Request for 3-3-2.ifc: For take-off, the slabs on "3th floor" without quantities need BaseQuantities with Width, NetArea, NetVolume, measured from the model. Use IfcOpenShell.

First a look at what the model holds.

```python
import ifcopenshell
import ifcopenshell.util.element
import ifcopenshell.util.unit

model = ifcopenshell.open("3-3-2.ifc")
print(model.schema)
for unit_type in ("LENGTHUNIT", "AREAUNIT", "VOLUMEUNIT"):
    print(unit_type, ifcopenshell.util.unit.calculate_unit_scale(model, unit_type))
storey = next(s for s in model.by_type("IfcBuildingStorey") if s.Name == "3th floor")
slabs = [e for e in ifcopenshell.util.element.get_decomposition(storey) if e.is_a("IfcSlab")]
for e in sorted(slabs, key=lambda e: e.id()):
    print(e.id(), e.is_a(), e.Name, list(ifcopenshell.util.element.get_psets(e, qtos_only=True)), sep=" | ")
```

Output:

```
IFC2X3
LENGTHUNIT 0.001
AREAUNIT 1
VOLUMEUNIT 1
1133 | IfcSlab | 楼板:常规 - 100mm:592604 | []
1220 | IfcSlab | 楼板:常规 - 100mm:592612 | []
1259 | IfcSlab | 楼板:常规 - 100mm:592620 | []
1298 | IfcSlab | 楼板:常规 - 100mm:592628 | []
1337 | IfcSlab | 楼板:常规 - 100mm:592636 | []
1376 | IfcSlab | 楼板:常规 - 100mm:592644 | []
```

```python
import ifcopenshell
import ifcopenshell.api.pset
import ifcopenshell.geom
import ifcopenshell.util.element
import ifcopenshell.util.shape
import ifcopenshell.util.unit

model = ifcopenshell.open("3-3-2.ifc")
unit_scale = ifcopenshell.util.unit.calculate_unit_scale(model)
area_scale = ifcopenshell.util.unit.calculate_unit_scale(model, "AREAUNIT")
volume_scale = ifcopenshell.util.unit.calculate_unit_scale(model, "VOLUMEUNIT")
settings = ifcopenshell.geom.settings()

storey = next(s for s in model.by_type("IfcBuildingStorey") if s.Name == "3th floor")
slabs = [e for e in ifcopenshell.util.element.get_decomposition(storey) if e.is_a("IfcSlab")]

for e in sorted(slabs, key=lambda e: e.id()):
    if ifcopenshell.util.element.get_psets(e, qtos_only=True, should_inherit=False):
        continue
    # Geometry comes back in metres, in the element's own axes.
    shape = ifcopenshell.geom.create_shape(settings, e)
    values = {
        "Width": ifcopenshell.util.shape.get_z(shape.geometry) / unit_scale,
        "NetArea": ifcopenshell.util.shape.get_footprint_area(shape.geometry) / area_scale,
        "NetVolume": ifcopenshell.util.shape.get_volume(shape.geometry) / volume_scale,
    }
    qto = ifcopenshell.api.pset.add_qto(model, product=e, name="BaseQuantities")
    ifcopenshell.api.pset.edit_qto(model, qto=qto, properties=values)
    print(e.id(), {k: round(v, 3) for k, v in values.items()})

model.write("3-3-2_rev.ifc")
```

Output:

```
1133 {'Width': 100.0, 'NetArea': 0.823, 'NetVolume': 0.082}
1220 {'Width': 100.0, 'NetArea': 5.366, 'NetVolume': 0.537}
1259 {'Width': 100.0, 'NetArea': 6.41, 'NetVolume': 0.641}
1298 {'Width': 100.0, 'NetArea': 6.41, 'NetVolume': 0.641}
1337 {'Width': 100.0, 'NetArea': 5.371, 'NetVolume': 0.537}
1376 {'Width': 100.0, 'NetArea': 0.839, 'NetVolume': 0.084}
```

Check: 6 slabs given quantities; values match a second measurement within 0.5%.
